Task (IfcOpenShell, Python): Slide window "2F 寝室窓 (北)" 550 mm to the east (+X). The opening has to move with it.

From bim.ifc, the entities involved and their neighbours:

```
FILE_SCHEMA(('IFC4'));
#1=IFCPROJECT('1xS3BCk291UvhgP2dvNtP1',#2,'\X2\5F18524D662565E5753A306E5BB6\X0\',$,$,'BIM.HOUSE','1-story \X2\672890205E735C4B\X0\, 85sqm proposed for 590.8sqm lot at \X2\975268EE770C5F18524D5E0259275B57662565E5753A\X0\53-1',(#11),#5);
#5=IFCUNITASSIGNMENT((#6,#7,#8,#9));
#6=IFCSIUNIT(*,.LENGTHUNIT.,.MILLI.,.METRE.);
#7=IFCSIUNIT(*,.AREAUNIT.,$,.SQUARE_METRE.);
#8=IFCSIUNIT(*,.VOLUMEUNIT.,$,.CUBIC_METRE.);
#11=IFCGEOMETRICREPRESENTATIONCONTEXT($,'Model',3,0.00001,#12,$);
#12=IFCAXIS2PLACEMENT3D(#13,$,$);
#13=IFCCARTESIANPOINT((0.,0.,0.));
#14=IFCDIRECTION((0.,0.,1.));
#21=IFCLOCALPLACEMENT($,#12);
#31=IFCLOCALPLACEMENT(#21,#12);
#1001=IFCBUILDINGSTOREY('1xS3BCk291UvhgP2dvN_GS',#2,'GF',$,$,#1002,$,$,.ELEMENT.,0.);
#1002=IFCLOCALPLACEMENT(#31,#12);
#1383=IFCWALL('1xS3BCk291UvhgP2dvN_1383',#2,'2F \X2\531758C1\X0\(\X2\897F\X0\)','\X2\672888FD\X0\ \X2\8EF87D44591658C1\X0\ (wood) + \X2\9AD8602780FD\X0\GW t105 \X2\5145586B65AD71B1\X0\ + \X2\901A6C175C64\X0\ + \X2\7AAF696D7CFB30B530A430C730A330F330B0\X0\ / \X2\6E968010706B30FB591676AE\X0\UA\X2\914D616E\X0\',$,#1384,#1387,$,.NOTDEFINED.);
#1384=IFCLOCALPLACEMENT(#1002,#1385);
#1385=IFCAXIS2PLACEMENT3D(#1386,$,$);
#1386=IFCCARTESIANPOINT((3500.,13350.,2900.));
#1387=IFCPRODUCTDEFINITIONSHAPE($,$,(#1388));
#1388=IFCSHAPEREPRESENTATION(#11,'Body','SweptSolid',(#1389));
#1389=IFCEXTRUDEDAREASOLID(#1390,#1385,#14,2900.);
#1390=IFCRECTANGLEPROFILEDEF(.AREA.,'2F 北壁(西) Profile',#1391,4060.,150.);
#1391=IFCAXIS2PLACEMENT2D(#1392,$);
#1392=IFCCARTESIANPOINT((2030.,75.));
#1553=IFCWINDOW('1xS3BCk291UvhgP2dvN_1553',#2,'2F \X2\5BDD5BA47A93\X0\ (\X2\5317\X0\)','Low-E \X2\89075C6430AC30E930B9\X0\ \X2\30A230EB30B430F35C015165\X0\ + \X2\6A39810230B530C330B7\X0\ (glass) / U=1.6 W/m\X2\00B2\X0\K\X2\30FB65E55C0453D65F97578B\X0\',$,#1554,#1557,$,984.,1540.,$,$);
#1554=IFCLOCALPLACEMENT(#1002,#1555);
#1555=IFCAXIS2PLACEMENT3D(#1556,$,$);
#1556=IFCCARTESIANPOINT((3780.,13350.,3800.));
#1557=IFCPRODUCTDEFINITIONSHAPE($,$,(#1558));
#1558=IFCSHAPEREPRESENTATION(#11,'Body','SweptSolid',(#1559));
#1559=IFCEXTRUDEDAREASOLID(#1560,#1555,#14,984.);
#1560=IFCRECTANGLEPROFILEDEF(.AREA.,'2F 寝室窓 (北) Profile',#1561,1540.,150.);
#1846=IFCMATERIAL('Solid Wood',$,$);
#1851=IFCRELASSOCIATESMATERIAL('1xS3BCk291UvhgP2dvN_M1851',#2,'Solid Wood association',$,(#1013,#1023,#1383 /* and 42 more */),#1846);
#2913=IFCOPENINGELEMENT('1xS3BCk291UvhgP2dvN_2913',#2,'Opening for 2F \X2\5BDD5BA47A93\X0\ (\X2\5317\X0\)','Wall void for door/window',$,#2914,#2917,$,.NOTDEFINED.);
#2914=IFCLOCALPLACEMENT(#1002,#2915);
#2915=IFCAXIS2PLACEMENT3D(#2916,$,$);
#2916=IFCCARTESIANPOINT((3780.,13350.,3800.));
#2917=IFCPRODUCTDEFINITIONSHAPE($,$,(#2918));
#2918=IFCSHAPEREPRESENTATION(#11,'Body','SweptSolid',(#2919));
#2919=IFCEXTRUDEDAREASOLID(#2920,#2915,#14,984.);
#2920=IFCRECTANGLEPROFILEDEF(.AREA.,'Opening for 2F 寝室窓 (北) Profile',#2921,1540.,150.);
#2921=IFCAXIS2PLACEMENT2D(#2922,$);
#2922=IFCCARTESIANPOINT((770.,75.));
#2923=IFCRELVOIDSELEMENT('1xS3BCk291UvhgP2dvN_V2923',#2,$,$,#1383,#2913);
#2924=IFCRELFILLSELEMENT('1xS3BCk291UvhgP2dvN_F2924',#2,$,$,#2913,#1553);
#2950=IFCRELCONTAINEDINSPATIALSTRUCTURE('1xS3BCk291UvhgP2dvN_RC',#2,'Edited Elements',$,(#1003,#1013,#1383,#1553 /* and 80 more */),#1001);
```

```python
import ifcopenshell
import ifcopenshell.api.geometry
import ifcopenshell.util.placement
import ifcopenshell.util.unit

model = ifcopenshell.open("bim.ifc")
unit_scale = ifcopenshell.util.unit.calculate_unit_scale(model)

window = model.by_guid("1xS3BCk291UvhgP2dvN_1553")
opening = window.FillsVoids[0].RelatingOpeningElement
wall = opening.VoidsElements[0].RelatingBuildingElement

wall_matrix = ifcopenshell.util.placement.get_local_placement(wall.ObjectPlacement)
shift = wall_matrix[:3, 0] * 0.55 / unit_scale
before = ifcopenshell.util.placement.get_local_placement(window.ObjectPlacement)[:3, 3].copy()

# The window is not placed relative to its opening, so move both.
for product in (opening, window):
    matrix = ifcopenshell.util.placement.get_local_placement(product.ObjectPlacement)
    matrix[:3, 3] += shift
    ifcopenshell.api.geometry.edit_object_placement(model, product=product, matrix=matrix, is_si=False)

after = ifcopenshell.util.placement.get_local_placement(window.ObjectPlacement)[:3, 3]
print("window moved by", (after - before).round(3) + 0.0)

model.write("bim_v2.ifc")
```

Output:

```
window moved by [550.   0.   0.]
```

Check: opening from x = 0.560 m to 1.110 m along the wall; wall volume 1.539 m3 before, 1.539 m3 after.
